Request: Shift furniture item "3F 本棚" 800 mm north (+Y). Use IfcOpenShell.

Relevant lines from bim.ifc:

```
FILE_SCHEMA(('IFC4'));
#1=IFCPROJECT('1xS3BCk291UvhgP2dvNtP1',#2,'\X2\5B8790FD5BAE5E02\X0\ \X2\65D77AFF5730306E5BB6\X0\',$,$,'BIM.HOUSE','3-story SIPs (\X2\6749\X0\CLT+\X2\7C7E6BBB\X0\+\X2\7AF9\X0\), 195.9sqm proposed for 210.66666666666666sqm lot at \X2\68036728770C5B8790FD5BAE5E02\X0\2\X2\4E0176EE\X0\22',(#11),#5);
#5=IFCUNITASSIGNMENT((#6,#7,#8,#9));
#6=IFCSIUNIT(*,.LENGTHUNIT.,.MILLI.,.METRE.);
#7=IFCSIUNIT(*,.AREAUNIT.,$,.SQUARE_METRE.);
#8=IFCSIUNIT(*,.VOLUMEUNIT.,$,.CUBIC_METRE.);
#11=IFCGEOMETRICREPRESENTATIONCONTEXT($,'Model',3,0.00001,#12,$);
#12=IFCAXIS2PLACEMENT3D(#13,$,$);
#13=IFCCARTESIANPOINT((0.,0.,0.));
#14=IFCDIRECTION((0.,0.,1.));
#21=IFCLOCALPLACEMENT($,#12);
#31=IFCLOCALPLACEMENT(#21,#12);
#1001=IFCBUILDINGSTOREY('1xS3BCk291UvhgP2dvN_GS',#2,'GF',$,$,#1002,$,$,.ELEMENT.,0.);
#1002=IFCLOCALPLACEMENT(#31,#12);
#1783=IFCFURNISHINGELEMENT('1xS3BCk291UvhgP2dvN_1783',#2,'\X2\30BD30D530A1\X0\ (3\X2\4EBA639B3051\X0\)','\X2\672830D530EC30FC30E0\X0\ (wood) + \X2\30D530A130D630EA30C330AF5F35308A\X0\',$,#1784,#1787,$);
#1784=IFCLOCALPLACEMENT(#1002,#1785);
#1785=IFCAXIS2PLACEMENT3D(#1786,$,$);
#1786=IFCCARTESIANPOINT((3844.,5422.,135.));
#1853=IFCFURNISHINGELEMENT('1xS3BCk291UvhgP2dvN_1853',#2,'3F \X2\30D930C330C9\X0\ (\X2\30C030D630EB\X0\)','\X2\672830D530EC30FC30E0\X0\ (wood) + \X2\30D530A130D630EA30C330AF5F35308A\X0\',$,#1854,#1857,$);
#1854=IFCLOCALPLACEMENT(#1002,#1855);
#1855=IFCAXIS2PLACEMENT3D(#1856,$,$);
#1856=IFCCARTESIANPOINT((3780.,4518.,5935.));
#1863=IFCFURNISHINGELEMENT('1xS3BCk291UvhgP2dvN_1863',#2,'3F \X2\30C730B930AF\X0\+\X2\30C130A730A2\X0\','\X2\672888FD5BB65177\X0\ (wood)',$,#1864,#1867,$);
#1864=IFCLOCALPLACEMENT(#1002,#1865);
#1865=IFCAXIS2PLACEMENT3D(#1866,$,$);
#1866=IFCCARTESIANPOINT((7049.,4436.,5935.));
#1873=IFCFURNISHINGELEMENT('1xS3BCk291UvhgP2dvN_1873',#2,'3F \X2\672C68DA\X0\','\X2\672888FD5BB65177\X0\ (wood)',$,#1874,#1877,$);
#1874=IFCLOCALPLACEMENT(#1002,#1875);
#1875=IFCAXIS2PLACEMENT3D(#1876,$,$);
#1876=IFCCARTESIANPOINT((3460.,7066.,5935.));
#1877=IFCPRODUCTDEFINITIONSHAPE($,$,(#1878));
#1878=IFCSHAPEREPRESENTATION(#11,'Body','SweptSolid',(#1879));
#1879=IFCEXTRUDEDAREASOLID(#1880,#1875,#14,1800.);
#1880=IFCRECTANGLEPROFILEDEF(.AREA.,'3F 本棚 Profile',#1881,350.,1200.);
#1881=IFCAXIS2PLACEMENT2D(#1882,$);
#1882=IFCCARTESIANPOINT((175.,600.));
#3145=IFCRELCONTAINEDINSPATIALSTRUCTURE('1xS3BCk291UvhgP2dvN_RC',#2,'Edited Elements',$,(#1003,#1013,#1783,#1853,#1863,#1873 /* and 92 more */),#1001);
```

```python
import ifcopenshell
import ifcopenshell.api.geometry
import ifcopenshell.util.placement

model = ifcopenshell.open("bim.ifc")

item = model.by_guid("1xS3BCk291UvhgP2dvN_1873")
matrix = ifcopenshell.util.placement.get_local_placement(item.ObjectPlacement)
matrix[1, 3] += 800.0
ifcopenshell.api.geometry.edit_object_placement(model, product=item, matrix=matrix, is_si=False)

print(ifcopenshell.util.placement.get_local_placement(item.ObjectPlacement).round(3) + 0.0)

model.write("bim_v2.ifc")
```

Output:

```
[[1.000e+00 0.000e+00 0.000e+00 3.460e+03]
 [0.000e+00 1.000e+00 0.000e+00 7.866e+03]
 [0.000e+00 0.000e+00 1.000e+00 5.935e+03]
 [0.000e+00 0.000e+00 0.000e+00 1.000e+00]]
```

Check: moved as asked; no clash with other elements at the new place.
